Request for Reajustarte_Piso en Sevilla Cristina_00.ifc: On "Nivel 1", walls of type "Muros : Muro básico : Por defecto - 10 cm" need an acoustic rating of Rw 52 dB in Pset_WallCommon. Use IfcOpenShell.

First a look at what the model holds.

```python
import ifcopenshell
import ifcopenshell.util.element

model = ifcopenshell.open("Reajustarte_Piso en Sevilla Cristina_00.ifc")
print(model.schema)
storey = next(s for s in model.by_type("IfcBuildingStorey") if s.Name == "Nivel 1")
walls = [e for e in ifcopenshell.util.element.get_decomposition(storey) if e.is_a("IfcWall")]
seen = {}
for e in walls:
    element_type = ifcopenshell.util.element.get_type(e)
    key = (element_type.Name if element_type != e and element_type else None, ifcopenshell.util.element.get_pset(e, "Pset_WallCommon", "AcousticRating"))
    seen[key] = seen.get(key, 0) + 1
for (name, value), count in sorted(seen.items(), key=str):
    print(count, "x", name, "|", value)
```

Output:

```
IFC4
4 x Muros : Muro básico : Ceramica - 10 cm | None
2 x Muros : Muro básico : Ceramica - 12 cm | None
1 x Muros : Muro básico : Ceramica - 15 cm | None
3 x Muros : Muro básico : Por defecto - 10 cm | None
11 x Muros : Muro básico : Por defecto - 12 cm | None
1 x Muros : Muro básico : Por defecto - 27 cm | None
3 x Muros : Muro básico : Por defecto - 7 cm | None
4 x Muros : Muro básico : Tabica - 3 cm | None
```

```python
import ifcopenshell
import ifcopenshell.api.pset
import ifcopenshell.util.element

model = ifcopenshell.open("Reajustarte_Piso en Sevilla Cristina_00.ifc")

storey = next(s for s in model.by_type("IfcBuildingStorey") if s.Name == "Nivel 1")
walls = [e for e in ifcopenshell.util.element.get_decomposition(storey) if e.is_a("IfcWall")]

count = 0
for e in walls:
    element_type = ifcopenshell.util.element.get_type(e)
    if element_type in (None, e) or element_type.Name != "Muros : Muro básico : Por defecto - 10 cm":
        continue
    # add_pset returns the element's existing set when there is one.
    pset = ifcopenshell.api.pset.add_pset(model, product=e, name="Pset_WallCommon")
    ifcopenshell.api.pset.edit_pset(model, pset=pset, properties={"AcousticRating": "Rw 52 dB"})
    count += 1

print(count, "walls updated")

model.write("Reajustarte_Piso en Sevilla Cristina_00_updated.ifc")
```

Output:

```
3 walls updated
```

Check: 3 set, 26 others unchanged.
